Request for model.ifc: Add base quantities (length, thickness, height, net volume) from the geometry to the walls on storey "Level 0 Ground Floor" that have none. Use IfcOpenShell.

First a look at what the model holds.

```python
import ifcopenshell
import ifcopenshell.util.element
import ifcopenshell.util.unit

model = ifcopenshell.open("model.ifc")
print(model.schema)
for unit_type in ("LENGTHUNIT", "AREAUNIT", "VOLUMEUNIT"):
    print(unit_type, ifcopenshell.util.unit.calculate_unit_scale(model, unit_type))
storey = next(s for s in model.by_type("IfcBuildingStorey") if s.Name == "Level 0 Ground Floor")
walls = [e for e in ifcopenshell.util.element.get_decomposition(storey) if e.is_a("IfcWall")]
for e in sorted(walls, key=lambda e: e.id()):
    print(e.id(), e.is_a(), e.Name, list(ifcopenshell.util.element.get_psets(e, qtos_only=True)), sep=" | ")
```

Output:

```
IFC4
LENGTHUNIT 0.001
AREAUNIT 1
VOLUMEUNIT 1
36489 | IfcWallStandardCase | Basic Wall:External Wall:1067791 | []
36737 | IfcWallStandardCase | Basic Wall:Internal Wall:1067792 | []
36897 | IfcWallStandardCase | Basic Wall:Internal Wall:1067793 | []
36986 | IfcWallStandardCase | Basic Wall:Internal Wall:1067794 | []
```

```python
import ifcopenshell
import ifcopenshell.api.pset
import ifcopenshell.geom
import ifcopenshell.util.element
import ifcopenshell.util.shape
import ifcopenshell.util.unit

model = ifcopenshell.open("model.ifc")
unit_scale = ifcopenshell.util.unit.calculate_unit_scale(model)
volume_scale = ifcopenshell.util.unit.calculate_unit_scale(model, "VOLUMEUNIT")
settings = ifcopenshell.geom.settings()

storey = next(s for s in model.by_type("IfcBuildingStorey") if s.Name == "Level 0 Ground Floor")
walls = [e for e in ifcopenshell.util.element.get_decomposition(storey) if e.is_a("IfcWall")]

for e in sorted(walls, key=lambda e: e.id()):
    if ifcopenshell.util.element.get_psets(e, qtos_only=True, should_inherit=False):
        continue
    # Geometry comes back in metres, in the element's own axes.
    shape = ifcopenshell.geom.create_shape(settings, e)
    values = {
        "Length": ifcopenshell.util.shape.get_x(shape.geometry) / unit_scale,
        "Width": ifcopenshell.util.shape.get_y(shape.geometry) / unit_scale,
        "Height": ifcopenshell.util.shape.get_z(shape.geometry) / unit_scale,
        "NetVolume": ifcopenshell.util.shape.get_volume(shape.geometry) / volume_scale,
    }
    qto = ifcopenshell.api.pset.add_qto(model, product=e, name="Qto_WallBaseQuantities")
    ifcopenshell.api.pset.edit_qto(model, qto=qto, properties=values)
    print(e.id(), {k: round(v, 3) for k, v in values.items()})

model.write("model-out.ifc")
```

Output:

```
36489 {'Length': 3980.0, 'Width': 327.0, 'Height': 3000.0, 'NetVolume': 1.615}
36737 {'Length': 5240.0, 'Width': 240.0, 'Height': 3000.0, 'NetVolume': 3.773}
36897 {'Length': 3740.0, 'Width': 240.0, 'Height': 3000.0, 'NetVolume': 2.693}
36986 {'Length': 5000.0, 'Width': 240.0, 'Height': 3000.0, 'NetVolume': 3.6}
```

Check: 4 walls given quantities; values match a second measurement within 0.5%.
